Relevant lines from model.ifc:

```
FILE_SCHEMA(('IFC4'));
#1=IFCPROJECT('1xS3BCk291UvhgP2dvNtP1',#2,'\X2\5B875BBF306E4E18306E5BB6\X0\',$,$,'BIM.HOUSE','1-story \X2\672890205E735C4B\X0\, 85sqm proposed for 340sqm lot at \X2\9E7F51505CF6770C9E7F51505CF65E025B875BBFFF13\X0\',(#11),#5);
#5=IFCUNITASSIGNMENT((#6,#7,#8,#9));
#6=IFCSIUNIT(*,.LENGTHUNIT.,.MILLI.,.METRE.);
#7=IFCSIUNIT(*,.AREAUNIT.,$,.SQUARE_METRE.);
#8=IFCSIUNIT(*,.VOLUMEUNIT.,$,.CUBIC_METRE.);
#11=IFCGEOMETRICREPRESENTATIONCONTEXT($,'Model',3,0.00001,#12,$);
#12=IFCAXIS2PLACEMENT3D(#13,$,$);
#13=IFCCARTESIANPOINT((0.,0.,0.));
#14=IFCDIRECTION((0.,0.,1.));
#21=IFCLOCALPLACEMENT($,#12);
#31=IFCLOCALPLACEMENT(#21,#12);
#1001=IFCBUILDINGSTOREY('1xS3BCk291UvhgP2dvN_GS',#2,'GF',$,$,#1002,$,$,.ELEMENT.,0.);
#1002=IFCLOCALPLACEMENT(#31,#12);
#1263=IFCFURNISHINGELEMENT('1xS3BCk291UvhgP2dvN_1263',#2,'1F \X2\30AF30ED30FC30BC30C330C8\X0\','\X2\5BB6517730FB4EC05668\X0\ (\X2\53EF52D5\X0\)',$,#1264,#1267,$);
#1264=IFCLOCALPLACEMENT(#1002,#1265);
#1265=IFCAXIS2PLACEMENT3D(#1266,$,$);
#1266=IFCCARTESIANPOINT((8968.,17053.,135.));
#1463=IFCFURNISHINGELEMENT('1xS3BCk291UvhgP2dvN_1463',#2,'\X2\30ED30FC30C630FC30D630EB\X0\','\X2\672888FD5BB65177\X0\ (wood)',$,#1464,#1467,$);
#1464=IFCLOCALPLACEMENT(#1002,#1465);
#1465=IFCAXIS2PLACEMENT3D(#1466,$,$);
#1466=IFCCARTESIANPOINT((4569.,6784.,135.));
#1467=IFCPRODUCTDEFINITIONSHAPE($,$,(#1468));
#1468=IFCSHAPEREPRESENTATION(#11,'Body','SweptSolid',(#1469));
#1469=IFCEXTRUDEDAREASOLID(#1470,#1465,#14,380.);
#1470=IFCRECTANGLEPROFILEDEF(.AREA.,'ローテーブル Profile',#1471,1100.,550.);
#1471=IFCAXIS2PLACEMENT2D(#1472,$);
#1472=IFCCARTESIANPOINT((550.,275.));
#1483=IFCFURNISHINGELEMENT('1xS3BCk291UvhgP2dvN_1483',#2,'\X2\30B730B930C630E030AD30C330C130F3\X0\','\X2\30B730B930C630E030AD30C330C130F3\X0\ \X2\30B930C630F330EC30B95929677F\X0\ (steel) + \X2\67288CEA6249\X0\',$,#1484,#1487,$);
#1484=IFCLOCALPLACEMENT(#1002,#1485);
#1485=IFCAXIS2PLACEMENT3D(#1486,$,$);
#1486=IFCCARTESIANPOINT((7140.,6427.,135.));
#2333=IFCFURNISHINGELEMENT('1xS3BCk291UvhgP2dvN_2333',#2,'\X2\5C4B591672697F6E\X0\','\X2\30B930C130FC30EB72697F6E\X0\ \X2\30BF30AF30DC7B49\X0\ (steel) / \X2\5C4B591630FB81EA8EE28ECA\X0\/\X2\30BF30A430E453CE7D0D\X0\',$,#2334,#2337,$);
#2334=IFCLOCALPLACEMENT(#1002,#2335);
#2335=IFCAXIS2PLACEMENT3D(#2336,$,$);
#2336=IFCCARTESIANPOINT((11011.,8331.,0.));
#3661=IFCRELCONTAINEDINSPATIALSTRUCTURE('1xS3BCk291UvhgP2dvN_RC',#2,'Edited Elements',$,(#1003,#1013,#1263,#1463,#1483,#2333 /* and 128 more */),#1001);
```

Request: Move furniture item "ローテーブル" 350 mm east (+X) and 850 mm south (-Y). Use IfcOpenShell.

```python
import ifcopenshell
import ifcopenshell.api.geometry
import ifcopenshell.util.placement
import ifcopenshell.util.unit

model = ifcopenshell.open("model.ifc")
unit_scale = ifcopenshell.util.unit.calculate_unit_scale(model)

item = model.by_guid("1xS3BCk291UvhgP2dvN_1463")
matrix = ifcopenshell.util.placement.get_local_placement(item.ObjectPlacement)
matrix[0, 3] += 0.35 / unit_scale
matrix[1, 3] -= 0.85 / unit_scale
ifcopenshell.api.geometry.edit_object_placement(model, product=item, matrix=matrix, is_si=False)

print(ifcopenshell.util.placement.get_local_placement(item.ObjectPlacement).round(3) + 0.0)

model.write("model_edited.ifc")
```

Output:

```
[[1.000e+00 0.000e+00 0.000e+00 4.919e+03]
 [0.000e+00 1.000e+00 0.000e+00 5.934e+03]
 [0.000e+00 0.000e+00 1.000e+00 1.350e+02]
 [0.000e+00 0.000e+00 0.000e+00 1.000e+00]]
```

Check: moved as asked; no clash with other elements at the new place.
